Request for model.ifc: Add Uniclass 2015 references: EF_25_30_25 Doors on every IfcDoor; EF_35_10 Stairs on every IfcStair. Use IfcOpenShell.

First a look at what the model holds.

```python
import ifcopenshell

model = ifcopenshell.open("model.ifc")
print(model.schema)
print("classifications:", [c.Name for c in model.by_type("IfcClassification")])
for ifc_class in ("IfcDoor", "IfcRoof", "IfcStair", "IfcWall", "IfcWindow"):
    print(ifc_class, len(model.by_type(ifc_class)))
```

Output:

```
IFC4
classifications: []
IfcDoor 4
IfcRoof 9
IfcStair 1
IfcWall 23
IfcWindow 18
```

```python
import ifcopenshell
import ifcopenshell.api.classification

model = ifcopenshell.open("model.ifc")

system = ifcopenshell.api.classification.add_classification(model, classification="Uniclass 2015")

codes = {
    "IfcDoor": ("EF_25_30_25", "Doors"),
    "IfcStair": ("EF_35_10", "Stairs"),
}
for ifc_class, (code, name) in codes.items():
    products = model.by_type(ifc_class)
    ifcopenshell.api.classification.add_reference(
        model, products=products, classification=system, identification=code, name=name
    )
    print(code, len(products))

model.write("model_updated.ifc")
```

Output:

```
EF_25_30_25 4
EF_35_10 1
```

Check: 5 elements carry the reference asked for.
